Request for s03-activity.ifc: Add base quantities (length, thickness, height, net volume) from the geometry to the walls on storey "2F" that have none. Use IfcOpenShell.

First a look at what the model holds.

```python
import ifcopenshell
import ifcopenshell.util.element
import ifcopenshell.util.unit

model = ifcopenshell.open("s03-activity.ifc")
print(model.schema)
for unit_type in ("LENGTHUNIT", "AREAUNIT", "VOLUMEUNIT"):
    print(unit_type, ifcopenshell.util.unit.calculate_unit_scale(model, unit_type))
storey = next(s for s in model.by_type("IfcBuildingStorey") if s.Name == "2F")
walls = [e for e in ifcopenshell.util.element.get_decomposition(storey) if e.is_a("IfcWall")]
for e in sorted(walls, key=lambda e: e.id()):
    print(e.id(), e.is_a(), e.Name, list(ifcopenshell.util.element.get_psets(e, qtos_only=True)), sep=" | ")
```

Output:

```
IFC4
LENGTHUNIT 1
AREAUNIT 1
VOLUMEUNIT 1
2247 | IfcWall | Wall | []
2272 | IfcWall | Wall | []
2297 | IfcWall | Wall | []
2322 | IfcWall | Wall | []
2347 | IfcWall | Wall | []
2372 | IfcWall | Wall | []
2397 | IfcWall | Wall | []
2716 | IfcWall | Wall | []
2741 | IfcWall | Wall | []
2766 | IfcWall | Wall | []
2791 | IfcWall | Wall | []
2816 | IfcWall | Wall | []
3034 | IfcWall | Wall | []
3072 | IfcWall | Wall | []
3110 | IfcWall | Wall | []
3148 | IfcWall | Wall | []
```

```python
import ifcopenshell
import ifcopenshell.api.pset
import ifcopenshell.geom
import ifcopenshell.util.element
import ifcopenshell.util.shape
import ifcopenshell.util.unit

model = ifcopenshell.open("s03-activity.ifc")
unit_scale = ifcopenshell.util.unit.calculate_unit_scale(model)
volume_scale = ifcopenshell.util.unit.calculate_unit_scale(model, "VOLUMEUNIT")
settings = ifcopenshell.geom.settings()

storey = next(s for s in model.by_type("IfcBuildingStorey") if s.Name == "2F")
walls = [e for e in ifcopenshell.util.element.get_decomposition(storey) if e.is_a("IfcWall")]

for e in sorted(walls, key=lambda e: e.id()):
    if ifcopenshell.util.element.get_psets(e, qtos_only=True, should_inherit=False):
        continue
    # Geometry comes back in metres, in the element's own axes.
    shape = ifcopenshell.geom.create_shape(settings, e)
    values = {
        "Length": ifcopenshell.util.shape.get_x(shape.geometry) / unit_scale,
        "Width": ifcopenshell.util.shape.get_y(shape.geometry) / unit_scale,
        "Height": ifcopenshell.util.shape.get_z(shape.geometry) / unit_scale,
        "NetVolume": ifcopenshell.util.shape.get_volume(shape.geometry) / volume_scale,
    }
    qto = ifcopenshell.api.pset.add_qto(model, product=e, name="Qto_WallBaseQuantities")
    ifcopenshell.api.pset.edit_qto(model, qto=qto, properties=values)
    print(e.id(), {k: round(v, 3) for k, v in values.items()})

model.write("s03-activity_updated.ifc")
```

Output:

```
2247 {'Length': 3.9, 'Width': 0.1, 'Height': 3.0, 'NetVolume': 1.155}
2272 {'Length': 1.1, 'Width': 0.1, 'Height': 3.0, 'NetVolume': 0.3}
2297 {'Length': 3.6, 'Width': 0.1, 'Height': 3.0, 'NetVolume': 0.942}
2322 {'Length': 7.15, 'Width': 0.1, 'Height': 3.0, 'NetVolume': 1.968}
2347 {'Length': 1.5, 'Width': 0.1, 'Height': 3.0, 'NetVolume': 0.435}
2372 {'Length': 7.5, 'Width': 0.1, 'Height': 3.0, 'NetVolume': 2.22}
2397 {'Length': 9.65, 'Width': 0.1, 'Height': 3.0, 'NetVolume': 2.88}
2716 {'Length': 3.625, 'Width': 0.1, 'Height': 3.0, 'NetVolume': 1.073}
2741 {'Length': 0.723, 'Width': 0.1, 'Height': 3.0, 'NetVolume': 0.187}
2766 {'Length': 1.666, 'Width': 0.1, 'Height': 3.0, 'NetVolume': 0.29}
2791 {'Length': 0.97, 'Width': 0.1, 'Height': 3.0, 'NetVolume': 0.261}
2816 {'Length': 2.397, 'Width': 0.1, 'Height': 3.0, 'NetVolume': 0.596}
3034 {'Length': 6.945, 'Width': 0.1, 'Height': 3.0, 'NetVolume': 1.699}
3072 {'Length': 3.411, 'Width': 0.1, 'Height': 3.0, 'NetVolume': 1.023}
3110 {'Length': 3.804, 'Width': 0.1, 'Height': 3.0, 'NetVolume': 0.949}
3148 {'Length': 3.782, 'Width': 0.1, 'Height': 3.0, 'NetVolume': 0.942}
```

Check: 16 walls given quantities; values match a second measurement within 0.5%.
